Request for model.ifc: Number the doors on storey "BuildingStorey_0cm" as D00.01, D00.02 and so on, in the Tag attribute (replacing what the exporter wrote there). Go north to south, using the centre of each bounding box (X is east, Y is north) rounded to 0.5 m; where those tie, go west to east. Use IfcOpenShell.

First a look at what the model holds.

```python
import ifcopenshell
import ifcopenshell.util.element
import ifcopenshell.util.placement

model = ifcopenshell.open("model.ifc")
print(model.schema)
storey = next(s for s in model.by_type("IfcBuildingStorey") if s.Name == "BuildingStorey_0cm")
doors = [e for e in ifcopenshell.util.element.get_decomposition(storey) if e.is_a("IfcDoor")]
for e in sorted(doors, key=lambda e: e.id()):
    origin = ifcopenshell.util.placement.get_local_placement(e.ObjectPlacement)[:3, 3]
    print(e.id(), e.Tag, e.Name, origin.round(2) + 0.0, sep=" | ")
```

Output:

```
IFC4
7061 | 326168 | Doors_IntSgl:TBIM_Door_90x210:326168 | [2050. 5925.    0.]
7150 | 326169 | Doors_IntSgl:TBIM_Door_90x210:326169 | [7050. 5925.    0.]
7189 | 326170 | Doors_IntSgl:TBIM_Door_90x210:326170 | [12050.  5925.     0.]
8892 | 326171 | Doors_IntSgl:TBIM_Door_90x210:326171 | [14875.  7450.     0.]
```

```python
import ifcopenshell
import ifcopenshell.geom
import ifcopenshell.util.element
import ifcopenshell.util.shape

model = ifcopenshell.open("model.ifc")
settings = ifcopenshell.geom.settings()
settings.set("use-world-coords", True)


def centre(element):
    shape = ifcopenshell.geom.create_shape(settings, element)
    return ifcopenshell.util.shape.get_bbox_centroid(shape.geometry)


storey = next(s for s in model.by_type("IfcBuildingStorey") if s.Name == "BuildingStorey_0cm")
doors = [e for e in ifcopenshell.util.element.get_decomposition(storey) if e.is_a("IfcDoor")]

# Insertion points can sit at a corner or the storey origin, so sort by the geometry (in metres).
centres = {e: centre(e) for e in doors}
doors.sort(key=lambda e: (-round(centres[e][1] / 0.5), centres[e][0]))

for i, e in enumerate(doors, start=1):
    number = f"D00.{i:02d}"
    e.Tag = number
    print(e.id(), number)

model.write("model_v2.ifc")
```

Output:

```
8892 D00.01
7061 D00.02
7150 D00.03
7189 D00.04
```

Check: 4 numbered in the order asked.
